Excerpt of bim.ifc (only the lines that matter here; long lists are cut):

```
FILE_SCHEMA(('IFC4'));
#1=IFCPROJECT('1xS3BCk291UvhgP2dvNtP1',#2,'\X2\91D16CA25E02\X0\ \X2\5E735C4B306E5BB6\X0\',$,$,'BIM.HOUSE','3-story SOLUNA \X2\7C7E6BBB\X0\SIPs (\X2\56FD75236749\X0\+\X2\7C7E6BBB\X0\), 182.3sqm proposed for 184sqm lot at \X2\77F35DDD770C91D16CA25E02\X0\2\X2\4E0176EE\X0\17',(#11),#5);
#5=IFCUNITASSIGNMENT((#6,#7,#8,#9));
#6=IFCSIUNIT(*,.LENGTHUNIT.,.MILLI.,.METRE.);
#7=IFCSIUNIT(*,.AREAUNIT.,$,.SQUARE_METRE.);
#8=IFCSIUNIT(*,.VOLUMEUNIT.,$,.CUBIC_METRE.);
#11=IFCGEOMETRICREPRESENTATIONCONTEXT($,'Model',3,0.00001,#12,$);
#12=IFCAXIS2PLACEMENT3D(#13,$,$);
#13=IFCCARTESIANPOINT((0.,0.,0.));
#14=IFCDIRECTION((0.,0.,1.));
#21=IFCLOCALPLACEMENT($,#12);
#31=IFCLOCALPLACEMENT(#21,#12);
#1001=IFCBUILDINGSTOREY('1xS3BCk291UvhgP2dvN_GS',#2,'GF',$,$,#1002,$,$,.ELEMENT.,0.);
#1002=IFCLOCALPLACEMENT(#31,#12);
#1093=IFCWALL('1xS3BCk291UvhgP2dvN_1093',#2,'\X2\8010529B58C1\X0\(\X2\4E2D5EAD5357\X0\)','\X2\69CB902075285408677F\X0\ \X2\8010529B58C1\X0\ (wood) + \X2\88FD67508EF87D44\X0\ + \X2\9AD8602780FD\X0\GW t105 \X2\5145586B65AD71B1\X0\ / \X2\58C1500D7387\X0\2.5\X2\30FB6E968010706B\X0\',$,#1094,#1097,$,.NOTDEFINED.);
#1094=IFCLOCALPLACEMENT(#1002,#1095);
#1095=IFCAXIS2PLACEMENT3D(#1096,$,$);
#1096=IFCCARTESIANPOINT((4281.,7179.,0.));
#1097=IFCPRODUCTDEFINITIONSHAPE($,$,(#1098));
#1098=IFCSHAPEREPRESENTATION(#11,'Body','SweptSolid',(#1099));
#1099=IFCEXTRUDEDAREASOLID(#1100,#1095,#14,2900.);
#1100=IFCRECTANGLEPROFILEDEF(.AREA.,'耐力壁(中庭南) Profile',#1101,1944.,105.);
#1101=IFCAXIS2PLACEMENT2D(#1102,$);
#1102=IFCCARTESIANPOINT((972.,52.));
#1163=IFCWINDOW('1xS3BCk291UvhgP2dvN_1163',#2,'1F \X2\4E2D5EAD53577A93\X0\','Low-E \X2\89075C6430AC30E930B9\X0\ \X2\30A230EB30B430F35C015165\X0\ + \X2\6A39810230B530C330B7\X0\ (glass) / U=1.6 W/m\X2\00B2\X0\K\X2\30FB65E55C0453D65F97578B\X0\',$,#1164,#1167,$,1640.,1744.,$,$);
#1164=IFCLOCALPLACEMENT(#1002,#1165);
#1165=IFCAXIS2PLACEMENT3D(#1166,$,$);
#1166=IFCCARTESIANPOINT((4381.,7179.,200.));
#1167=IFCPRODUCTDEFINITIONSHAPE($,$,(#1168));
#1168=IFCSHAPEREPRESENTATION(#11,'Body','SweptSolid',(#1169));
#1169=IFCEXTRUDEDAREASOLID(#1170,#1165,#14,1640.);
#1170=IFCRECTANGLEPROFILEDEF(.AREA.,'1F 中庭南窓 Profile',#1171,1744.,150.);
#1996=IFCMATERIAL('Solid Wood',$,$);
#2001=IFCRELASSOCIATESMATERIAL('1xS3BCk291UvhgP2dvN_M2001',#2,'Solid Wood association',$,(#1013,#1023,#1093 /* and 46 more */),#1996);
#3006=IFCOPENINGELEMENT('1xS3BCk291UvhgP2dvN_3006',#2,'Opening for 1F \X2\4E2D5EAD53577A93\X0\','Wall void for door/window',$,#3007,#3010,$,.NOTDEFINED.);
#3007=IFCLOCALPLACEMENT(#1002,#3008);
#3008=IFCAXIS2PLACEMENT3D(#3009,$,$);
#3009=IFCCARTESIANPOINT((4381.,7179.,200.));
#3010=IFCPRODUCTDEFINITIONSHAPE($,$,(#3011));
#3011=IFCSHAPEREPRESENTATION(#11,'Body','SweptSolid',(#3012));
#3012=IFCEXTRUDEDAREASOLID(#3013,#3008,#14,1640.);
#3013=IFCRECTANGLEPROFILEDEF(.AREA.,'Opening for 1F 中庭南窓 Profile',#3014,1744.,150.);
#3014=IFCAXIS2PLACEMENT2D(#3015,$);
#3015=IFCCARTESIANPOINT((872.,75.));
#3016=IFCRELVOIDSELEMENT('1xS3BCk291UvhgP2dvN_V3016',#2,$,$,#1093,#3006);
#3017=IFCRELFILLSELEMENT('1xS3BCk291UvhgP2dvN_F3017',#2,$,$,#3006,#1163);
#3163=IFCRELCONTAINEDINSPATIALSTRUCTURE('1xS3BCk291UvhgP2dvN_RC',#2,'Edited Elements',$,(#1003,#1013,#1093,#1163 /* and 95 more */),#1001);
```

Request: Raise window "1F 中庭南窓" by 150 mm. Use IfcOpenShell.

```python
import numpy as np
import ifcopenshell
import ifcopenshell.api.geometry
import ifcopenshell.util.placement
import ifcopenshell.util.unit

model = ifcopenshell.open("bim.ifc")
unit_scale = ifcopenshell.util.unit.calculate_unit_scale(model)

window = model.by_id(1163)
opening = window.FillsVoids[0].RelatingOpeningElement
dz = 150.0

shift = np.array([0.0, 0.0, dz])
# The window is not placed relative to its opening, so move both.
for product in (opening, window):
    matrix = ifcopenshell.util.placement.get_local_placement(product.ObjectPlacement)
    matrix[:3, 3] += shift
    ifcopenshell.api.geometry.edit_object_placement(model, product=product, matrix=matrix, is_si=False)

print(f"moved by {dz * unit_scale:+.3f} m")

model.write("bim_updated.ifc")
```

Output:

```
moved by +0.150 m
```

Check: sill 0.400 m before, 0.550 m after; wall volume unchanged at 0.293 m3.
